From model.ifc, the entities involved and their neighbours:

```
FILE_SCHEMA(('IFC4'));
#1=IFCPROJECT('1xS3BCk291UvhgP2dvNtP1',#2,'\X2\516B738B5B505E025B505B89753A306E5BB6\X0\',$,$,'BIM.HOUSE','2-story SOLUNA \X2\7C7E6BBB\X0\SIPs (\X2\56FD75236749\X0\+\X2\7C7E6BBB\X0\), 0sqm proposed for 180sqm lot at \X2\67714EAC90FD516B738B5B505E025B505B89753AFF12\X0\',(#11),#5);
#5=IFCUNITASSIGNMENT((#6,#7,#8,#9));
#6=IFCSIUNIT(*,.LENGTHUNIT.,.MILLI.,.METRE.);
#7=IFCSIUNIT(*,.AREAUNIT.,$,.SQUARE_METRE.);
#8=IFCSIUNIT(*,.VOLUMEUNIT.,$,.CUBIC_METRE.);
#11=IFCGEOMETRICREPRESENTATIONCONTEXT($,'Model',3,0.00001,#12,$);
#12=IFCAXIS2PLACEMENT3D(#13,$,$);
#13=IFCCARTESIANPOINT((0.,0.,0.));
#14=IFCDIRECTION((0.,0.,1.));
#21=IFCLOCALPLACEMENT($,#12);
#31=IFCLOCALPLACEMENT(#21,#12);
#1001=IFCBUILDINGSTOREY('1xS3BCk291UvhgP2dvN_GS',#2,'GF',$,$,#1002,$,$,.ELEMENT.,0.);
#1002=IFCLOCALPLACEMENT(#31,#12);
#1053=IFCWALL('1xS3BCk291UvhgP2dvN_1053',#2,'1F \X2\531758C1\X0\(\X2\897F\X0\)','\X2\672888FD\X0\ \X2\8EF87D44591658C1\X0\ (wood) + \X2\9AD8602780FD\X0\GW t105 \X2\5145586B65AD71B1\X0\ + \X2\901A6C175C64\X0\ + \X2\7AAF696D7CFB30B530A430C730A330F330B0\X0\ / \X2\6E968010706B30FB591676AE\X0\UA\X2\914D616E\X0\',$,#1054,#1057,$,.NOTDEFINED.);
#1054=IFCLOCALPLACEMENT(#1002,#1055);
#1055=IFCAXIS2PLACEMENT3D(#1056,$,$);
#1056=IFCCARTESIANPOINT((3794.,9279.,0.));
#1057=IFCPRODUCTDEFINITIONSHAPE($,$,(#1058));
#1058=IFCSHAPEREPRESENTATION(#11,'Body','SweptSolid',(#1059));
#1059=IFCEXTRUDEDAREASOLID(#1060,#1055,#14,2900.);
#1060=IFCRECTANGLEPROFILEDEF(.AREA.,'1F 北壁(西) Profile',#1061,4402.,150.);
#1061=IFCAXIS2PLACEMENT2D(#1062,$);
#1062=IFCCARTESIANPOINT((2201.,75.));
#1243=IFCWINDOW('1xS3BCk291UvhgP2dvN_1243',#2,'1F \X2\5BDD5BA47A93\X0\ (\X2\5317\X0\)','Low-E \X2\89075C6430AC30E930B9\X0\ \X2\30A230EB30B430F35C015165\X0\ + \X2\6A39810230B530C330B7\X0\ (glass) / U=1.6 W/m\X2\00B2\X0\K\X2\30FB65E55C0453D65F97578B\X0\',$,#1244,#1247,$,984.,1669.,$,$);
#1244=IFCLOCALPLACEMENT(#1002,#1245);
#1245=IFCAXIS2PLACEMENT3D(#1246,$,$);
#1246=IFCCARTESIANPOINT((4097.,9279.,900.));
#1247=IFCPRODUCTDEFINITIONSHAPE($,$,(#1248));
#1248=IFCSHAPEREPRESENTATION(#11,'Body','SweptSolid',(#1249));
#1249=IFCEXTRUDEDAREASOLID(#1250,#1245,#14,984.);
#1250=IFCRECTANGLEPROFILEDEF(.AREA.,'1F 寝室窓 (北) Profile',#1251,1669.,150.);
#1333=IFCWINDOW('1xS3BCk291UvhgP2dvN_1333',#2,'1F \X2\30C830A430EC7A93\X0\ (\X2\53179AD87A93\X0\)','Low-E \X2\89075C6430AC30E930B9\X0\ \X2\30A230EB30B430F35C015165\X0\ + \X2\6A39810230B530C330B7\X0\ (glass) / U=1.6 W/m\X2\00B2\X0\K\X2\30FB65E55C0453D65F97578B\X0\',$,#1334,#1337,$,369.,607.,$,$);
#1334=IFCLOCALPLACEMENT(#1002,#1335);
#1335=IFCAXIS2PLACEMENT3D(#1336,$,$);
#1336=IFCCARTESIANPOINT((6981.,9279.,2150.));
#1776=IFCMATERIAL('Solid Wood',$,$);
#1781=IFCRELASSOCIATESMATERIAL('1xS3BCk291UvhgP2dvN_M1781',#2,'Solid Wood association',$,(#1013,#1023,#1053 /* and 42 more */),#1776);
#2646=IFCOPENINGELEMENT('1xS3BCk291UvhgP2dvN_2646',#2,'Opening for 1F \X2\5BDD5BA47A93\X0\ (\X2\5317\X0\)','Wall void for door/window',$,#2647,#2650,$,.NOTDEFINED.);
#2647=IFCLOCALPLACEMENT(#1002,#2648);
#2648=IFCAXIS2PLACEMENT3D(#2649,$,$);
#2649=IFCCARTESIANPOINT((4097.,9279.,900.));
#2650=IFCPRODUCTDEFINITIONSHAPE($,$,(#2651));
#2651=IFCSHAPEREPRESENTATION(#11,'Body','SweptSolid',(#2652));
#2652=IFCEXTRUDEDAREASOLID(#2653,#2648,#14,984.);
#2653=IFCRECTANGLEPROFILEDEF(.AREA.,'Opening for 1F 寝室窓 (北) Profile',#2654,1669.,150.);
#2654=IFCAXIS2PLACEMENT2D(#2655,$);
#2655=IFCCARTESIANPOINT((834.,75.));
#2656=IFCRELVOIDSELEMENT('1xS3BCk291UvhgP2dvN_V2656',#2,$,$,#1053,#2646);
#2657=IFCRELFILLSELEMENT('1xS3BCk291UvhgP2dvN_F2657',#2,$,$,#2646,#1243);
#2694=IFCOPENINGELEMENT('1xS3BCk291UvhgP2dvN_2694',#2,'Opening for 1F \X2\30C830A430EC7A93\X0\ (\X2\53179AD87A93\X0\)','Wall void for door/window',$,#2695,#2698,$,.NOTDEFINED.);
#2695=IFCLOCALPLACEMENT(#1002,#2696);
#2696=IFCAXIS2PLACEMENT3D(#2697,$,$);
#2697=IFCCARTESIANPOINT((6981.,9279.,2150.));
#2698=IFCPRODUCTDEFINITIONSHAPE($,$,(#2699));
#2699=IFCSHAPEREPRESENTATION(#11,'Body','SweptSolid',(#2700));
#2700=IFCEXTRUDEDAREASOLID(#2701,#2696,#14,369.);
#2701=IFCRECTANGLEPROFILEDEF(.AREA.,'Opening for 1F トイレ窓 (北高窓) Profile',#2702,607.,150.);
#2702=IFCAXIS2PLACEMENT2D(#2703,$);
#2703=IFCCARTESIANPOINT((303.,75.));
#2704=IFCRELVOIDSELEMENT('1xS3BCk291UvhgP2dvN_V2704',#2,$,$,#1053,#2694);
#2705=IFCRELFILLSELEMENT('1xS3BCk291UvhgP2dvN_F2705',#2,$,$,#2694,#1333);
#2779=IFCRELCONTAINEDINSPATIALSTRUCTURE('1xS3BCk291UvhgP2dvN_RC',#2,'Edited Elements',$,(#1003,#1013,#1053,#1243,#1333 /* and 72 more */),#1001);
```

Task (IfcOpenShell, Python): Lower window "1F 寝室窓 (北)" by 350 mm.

```python
import numpy as np
import ifcopenshell
import ifcopenshell.api.geometry
import ifcopenshell.util.placement
import ifcopenshell.util.unit

model = ifcopenshell.open("model.ifc")
unit_scale = ifcopenshell.util.unit.calculate_unit_scale(model)

window = model.by_id(1243)
opening = window.FillsVoids[0].RelatingOpeningElement
dz = -0.35 / unit_scale

shift = np.array([0.0, 0.0, dz])
# The window is not placed relative to its opening, so move both.
for product in (opening, window):
    matrix = ifcopenshell.util.placement.get_local_placement(product.ObjectPlacement)
    matrix[:3, 3] += shift
    ifcopenshell.api.geometry.edit_object_placement(model, product=product, matrix=matrix, is_si=False)

print(f"moved by {dz * unit_scale:+.3f} m")

model.write("model-out.ifc")
```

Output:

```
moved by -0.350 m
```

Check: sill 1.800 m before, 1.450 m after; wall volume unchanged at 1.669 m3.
